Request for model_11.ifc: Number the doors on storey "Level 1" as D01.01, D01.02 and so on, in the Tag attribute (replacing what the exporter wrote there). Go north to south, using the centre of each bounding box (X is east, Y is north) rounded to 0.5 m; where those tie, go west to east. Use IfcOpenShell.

First a look at what the model holds.

```python
import ifcopenshell
import ifcopenshell.util.element
import ifcopenshell.util.placement

model = ifcopenshell.open("model_11.ifc")
print(model.schema)
storey = next(s for s in model.by_type("IfcBuildingStorey") if s.Name == "Level 1")
doors = [e for e in ifcopenshell.util.element.get_decomposition(storey) if e.is_a("IfcDoor")]
for e in sorted(doors, key=lambda e: e.id()):
    origin = ifcopenshell.util.placement.get_local_placement(e.ObjectPlacement)[:3, 3]
    print(e.id(), e.Tag, e.Name, origin.round(2) + 0.0, sep=" | ")
```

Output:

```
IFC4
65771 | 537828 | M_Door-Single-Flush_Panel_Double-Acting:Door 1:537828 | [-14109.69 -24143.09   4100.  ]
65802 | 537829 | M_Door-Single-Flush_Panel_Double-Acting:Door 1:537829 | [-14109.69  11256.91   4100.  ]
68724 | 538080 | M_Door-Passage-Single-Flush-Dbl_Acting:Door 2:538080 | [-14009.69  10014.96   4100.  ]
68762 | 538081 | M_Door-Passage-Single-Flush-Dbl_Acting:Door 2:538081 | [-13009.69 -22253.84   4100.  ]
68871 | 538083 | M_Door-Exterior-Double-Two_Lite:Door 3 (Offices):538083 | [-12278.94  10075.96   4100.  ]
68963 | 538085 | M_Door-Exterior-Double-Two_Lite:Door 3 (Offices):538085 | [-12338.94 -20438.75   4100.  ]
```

```python
import ifcopenshell
import ifcopenshell.geom
import ifcopenshell.util.element
import ifcopenshell.util.shape

model = ifcopenshell.open("model_11.ifc")
settings = ifcopenshell.geom.settings()
settings.set("use-world-coords", True)


def centre(element):
    shape = ifcopenshell.geom.create_shape(settings, element)
    return ifcopenshell.util.shape.get_bbox_centroid(shape.geometry)


storey = next(s for s in model.by_type("IfcBuildingStorey") if s.Name == "Level 1")
doors = [e for e in ifcopenshell.util.element.get_decomposition(storey) if e.is_a("IfcDoor")]

# Insertion points can sit at a corner or the storey origin, so sort by the geometry (in metres).
centres = {e: centre(e) for e in doors}
doors.sort(key=lambda e: (-round(centres[e][1] / 0.5), centres[e][0]))

for i, e in enumerate(doors, start=1):
    number = f"D01.{i:02d}"
    e.Tag = number
    print(e.id(), number)

model.write("model_11_rev.ifc")
```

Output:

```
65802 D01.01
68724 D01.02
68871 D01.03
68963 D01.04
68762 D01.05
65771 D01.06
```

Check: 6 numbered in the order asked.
